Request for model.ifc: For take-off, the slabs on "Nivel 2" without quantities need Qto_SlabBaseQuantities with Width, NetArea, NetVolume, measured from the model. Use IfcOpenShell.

First a look at what the model holds.

```python
import ifcopenshell
import ifcopenshell.util.element
import ifcopenshell.util.unit

model = ifcopenshell.open("model.ifc")
print(model.schema)
for unit_type in ("LENGTHUNIT", "AREAUNIT", "VOLUMEUNIT"):
    print(unit_type, ifcopenshell.util.unit.calculate_unit_scale(model, unit_type))
storey = next(s for s in model.by_type("IfcBuildingStorey") if s.Name == "Nivel 2")
slabs = [e for e in ifcopenshell.util.element.get_decomposition(storey) if e.is_a("IfcSlab")]
for e in sorted(slabs, key=lambda e: e.id()):
    print(e.id(), e.is_a(), e.Name, list(ifcopenshell.util.element.get_psets(e, qtos_only=True)), sep=" | ")
```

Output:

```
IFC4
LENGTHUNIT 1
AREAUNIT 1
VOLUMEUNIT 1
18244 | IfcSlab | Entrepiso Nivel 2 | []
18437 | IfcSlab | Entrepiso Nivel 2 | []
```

```python
import ifcopenshell
import ifcopenshell.api.pset
import ifcopenshell.geom
import ifcopenshell.util.element
import ifcopenshell.util.shape
import ifcopenshell.util.unit

model = ifcopenshell.open("model.ifc")
unit_scale = ifcopenshell.util.unit.calculate_unit_scale(model)
area_scale = ifcopenshell.util.unit.calculate_unit_scale(model, "AREAUNIT")
volume_scale = ifcopenshell.util.unit.calculate_unit_scale(model, "VOLUMEUNIT")
settings = ifcopenshell.geom.settings()

storey = next(s for s in model.by_type("IfcBuildingStorey") if s.Name == "Nivel 2")
slabs = [e for e in ifcopenshell.util.element.get_decomposition(storey) if e.is_a("IfcSlab")]

for e in sorted(slabs, key=lambda e: e.id()):
    if ifcopenshell.util.element.get_psets(e, qtos_only=True, should_inherit=False):
        continue
    # Geometry comes back in metres, in the element's own axes.
    shape = ifcopenshell.geom.create_shape(settings, e)
    values = {
        "Width": ifcopenshell.util.shape.get_z(shape.geometry) / unit_scale,
        "NetArea": ifcopenshell.util.shape.get_footprint_area(shape.geometry) / area_scale,
        "NetVolume": ifcopenshell.util.shape.get_volume(shape.geometry) / volume_scale,
    }
    qto = ifcopenshell.api.pset.add_qto(model, product=e, name="Qto_SlabBaseQuantities")
    ifcopenshell.api.pset.edit_qto(model, qto=qto, properties=values)
    print(e.id(), {k: round(v, 3) for k, v in values.items()})

model.write("model_v2.ifc")
```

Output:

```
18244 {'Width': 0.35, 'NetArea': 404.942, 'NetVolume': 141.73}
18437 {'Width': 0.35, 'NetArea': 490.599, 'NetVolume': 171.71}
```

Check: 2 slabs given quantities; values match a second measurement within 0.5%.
